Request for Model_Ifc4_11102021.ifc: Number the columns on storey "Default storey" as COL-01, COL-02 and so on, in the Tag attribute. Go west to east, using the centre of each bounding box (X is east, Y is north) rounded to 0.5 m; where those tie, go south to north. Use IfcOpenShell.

First a look at what the model holds.

```python
import ifcopenshell
import ifcopenshell.util.element
import ifcopenshell.util.placement

model = ifcopenshell.open("Model_Ifc4_11102021.ifc")
print(model.schema)
storey = next(s for s in model.by_type("IfcBuildingStorey") if s.Name == "Default storey")
columns = [e for e in ifcopenshell.util.element.get_decomposition(storey) if e.is_a("IfcColumn")]
for e in sorted(columns, key=lambda e: e.id()):
    origin = ifcopenshell.util.placement.get_local_placement(e.ObjectPlacement)[:3, 3]
    print(e.id(), e.Tag, e.Name, origin.round(2) + 0.0, sep=" | ")
```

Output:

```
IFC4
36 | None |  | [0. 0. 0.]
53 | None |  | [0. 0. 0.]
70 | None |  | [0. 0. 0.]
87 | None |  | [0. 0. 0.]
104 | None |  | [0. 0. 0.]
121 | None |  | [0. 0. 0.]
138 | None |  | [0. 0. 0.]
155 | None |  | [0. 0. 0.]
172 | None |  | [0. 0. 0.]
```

```python
import ifcopenshell
import ifcopenshell.geom
import ifcopenshell.util.element
import ifcopenshell.util.shape

model = ifcopenshell.open("Model_Ifc4_11102021.ifc")
settings = ifcopenshell.geom.settings()
settings.set("use-world-coords", True)


def centre(element):
    shape = ifcopenshell.geom.create_shape(settings, element)
    return ifcopenshell.util.shape.get_bbox_centroid(shape.geometry)


storey = next(s for s in model.by_type("IfcBuildingStorey") if s.Name == "Default storey")
columns = [e for e in ifcopenshell.util.element.get_decomposition(storey) if e.is_a("IfcColumn")]

# Insertion points can sit at a corner or the storey origin, so sort by the geometry (in metres).
centres = {e: centre(e) for e in columns}
columns.sort(key=lambda e: (round(centres[e][0] / 0.5), centres[e][1]))

for i, e in enumerate(columns, start=1):
    number = f"COL-{i:02d}"
    e.Tag = number
    print(e.id(), number)

model.write("Model_Ifc4_11102021-out.ifc")
```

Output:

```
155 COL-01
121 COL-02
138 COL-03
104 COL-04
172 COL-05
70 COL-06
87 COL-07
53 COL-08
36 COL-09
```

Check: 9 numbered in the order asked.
